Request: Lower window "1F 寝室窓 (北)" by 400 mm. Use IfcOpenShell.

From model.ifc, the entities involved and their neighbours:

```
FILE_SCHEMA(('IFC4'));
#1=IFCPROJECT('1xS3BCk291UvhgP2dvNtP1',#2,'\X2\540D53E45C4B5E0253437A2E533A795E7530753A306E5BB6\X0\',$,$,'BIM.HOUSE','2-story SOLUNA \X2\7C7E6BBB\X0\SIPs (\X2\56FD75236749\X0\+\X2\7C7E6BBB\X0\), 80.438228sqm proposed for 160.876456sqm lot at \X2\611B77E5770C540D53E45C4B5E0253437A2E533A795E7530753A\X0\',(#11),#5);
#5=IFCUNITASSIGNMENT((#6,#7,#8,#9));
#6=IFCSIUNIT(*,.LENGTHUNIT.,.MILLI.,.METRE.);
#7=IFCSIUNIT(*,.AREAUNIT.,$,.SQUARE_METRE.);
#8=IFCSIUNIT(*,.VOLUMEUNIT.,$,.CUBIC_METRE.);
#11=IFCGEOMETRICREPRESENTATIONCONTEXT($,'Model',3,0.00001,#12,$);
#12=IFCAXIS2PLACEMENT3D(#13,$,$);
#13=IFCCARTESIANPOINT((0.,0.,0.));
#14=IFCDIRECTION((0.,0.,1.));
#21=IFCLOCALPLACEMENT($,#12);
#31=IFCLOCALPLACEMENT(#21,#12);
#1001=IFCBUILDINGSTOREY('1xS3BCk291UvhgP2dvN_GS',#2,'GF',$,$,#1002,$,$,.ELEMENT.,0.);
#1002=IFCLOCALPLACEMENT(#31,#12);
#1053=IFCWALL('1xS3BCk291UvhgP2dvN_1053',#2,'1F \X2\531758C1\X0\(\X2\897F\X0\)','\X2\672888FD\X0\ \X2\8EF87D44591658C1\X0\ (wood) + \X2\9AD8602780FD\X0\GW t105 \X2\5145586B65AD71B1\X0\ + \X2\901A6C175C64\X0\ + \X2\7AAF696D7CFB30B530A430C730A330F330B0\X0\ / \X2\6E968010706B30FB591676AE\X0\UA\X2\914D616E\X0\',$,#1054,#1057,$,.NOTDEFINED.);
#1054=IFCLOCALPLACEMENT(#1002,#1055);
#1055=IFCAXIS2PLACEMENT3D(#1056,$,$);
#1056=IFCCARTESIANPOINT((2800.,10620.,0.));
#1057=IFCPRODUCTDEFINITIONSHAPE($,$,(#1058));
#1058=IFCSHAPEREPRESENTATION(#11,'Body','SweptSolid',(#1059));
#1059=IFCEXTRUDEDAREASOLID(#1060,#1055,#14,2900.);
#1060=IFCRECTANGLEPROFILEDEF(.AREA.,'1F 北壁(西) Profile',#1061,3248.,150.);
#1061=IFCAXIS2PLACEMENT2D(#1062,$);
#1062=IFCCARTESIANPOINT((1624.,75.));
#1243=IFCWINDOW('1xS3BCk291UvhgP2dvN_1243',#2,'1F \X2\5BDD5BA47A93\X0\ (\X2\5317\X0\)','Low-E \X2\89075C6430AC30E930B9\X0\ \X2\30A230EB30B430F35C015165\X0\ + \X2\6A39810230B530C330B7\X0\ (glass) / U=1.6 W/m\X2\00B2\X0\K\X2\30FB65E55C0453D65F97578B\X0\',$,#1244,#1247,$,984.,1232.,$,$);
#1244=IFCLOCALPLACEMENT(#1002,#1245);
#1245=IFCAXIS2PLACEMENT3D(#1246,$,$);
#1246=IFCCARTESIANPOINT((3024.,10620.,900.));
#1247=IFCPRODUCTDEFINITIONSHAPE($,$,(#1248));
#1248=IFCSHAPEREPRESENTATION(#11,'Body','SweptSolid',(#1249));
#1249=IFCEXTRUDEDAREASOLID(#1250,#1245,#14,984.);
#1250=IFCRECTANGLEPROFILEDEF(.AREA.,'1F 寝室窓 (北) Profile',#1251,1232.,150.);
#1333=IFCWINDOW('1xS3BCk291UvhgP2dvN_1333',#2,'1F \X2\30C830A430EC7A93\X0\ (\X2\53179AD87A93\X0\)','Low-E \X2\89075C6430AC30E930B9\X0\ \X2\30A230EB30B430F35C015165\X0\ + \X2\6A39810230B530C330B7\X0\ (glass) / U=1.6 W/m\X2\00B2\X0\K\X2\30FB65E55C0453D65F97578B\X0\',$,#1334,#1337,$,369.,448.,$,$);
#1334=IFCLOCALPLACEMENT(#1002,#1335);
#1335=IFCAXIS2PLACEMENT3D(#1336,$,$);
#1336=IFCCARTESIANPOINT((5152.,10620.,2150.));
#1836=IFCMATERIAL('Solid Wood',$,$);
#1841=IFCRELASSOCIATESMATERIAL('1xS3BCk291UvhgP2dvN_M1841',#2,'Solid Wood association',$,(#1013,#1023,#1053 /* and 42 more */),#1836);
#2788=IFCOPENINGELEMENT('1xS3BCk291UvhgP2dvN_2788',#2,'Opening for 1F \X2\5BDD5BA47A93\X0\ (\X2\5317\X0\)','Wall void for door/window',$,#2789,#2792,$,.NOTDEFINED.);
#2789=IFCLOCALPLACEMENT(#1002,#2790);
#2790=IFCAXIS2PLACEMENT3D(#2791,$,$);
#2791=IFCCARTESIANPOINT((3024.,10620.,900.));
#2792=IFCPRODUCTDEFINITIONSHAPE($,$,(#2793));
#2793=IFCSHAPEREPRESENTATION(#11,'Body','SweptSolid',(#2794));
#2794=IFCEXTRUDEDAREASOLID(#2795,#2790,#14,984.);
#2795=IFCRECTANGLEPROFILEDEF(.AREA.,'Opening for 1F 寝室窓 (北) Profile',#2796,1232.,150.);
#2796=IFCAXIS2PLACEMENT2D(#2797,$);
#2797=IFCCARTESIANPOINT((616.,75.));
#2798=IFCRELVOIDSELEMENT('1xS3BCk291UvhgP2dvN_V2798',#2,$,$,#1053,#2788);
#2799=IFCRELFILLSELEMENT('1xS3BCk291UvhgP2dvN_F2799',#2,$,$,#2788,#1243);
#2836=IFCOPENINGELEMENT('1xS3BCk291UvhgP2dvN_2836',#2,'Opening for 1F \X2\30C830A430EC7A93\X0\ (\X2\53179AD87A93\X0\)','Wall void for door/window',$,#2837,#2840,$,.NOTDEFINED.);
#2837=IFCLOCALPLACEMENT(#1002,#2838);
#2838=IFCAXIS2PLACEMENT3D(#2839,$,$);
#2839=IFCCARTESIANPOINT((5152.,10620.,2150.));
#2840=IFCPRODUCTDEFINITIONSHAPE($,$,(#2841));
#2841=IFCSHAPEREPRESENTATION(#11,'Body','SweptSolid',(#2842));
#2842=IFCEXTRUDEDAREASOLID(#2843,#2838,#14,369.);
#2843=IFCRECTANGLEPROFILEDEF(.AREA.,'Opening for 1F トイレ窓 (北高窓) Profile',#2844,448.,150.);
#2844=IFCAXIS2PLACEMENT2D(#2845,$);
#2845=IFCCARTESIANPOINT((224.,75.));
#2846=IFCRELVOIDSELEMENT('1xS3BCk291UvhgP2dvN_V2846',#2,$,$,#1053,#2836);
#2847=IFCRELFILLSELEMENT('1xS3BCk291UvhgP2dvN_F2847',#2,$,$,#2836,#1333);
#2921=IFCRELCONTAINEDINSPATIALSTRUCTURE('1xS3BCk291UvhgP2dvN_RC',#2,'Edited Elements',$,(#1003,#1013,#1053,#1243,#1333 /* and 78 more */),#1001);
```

```python
import numpy as np
import ifcopenshell
import ifcopenshell.api.geometry
import ifcopenshell.util.placement
import ifcopenshell.util.unit

model = ifcopenshell.open("model.ifc")
unit_scale = ifcopenshell.util.unit.calculate_unit_scale(model)

window = model.by_id(1243)
opening = window.FillsVoids[0].RelatingOpeningElement
dz = -400.0

shift = np.array([0.0, 0.0, dz])
# The window is not placed relative to its opening, so move both.
for product in (opening, window):
    matrix = ifcopenshell.util.placement.get_local_placement(product.ObjectPlacement)
    matrix[:3, 3] += shift
    ifcopenshell.api.geometry.edit_object_placement(model, product=product, matrix=matrix, is_si=False)

print(f"moved by {dz * unit_scale:+.3f} m")

model.write("model-out.ifc")
```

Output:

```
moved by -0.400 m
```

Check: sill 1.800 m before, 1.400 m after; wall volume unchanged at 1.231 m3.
